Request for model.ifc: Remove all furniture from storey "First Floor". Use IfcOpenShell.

First a look at what the model holds.

```python
import ifcopenshell
import ifcopenshell.util.element

model = ifcopenshell.open("model.ifc")
print(model.schema)
storey = next(s for s in model.by_type("IfcBuildingStorey") if s.Name == "First Floor")
furniture = [e for e in ifcopenshell.util.element.get_decomposition(storey) if e.is_a("IfcFurnishingElement")]
seen = {}
for e in furniture:
    element_type = ifcopenshell.util.element.get_type(e)
    name = element_type.Name if element_type not in (None, e) else None
    seen[name] = seen.get(name, 0) + 1
for name, count in sorted(seen.items(), key=str):
    print(count, "x", name)
```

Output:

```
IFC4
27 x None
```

```python
import ifcopenshell
import ifcopenshell.api.root
import ifcopenshell.util.element

model = ifcopenshell.open("model.ifc")

storey = next(s for s in model.by_type("IfcBuildingStorey") if s.Name == "First Floor")
furniture = [e for e in ifcopenshell.util.element.get_decomposition(storey) if e.is_a("IfcFurnishingElement")]

for e in furniture:
    ifcopenshell.api.root.remove_product(model, product=e)
print(len(furniture), "removed")

model.write("model_edited.ifc")
```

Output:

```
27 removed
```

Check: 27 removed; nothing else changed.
